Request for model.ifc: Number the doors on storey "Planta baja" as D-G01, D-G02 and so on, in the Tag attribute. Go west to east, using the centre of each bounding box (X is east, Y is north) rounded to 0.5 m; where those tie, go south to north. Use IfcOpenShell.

First a look at what the model holds.

```python
import ifcopenshell
import ifcopenshell.util.element
import ifcopenshell.util.placement

model = ifcopenshell.open("model.ifc")
print(model.schema)
storey = next(s for s in model.by_type("IfcBuildingStorey") if s.Name == "Planta baja")
doors = [e for e in ifcopenshell.util.element.get_decomposition(storey) if e.is_a("IfcDoor")]
for e in sorted(doors, key=lambda e: e.id()):
    origin = ifcopenshell.util.placement.get_local_placement(e.ObjectPlacement)[:3, 3]
    print(e.id(), e.Tag, e.Name, origin.round(2) + 0.0, sep=" | ")
```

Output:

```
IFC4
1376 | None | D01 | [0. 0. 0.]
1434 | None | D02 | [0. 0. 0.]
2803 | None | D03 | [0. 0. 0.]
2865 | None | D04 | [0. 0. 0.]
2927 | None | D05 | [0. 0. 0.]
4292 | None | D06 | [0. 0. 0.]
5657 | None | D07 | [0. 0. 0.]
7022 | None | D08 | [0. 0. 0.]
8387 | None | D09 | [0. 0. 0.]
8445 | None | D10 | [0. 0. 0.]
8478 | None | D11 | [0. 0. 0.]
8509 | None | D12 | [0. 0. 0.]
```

```python
import ifcopenshell
import ifcopenshell.geom
import ifcopenshell.util.element
import ifcopenshell.util.shape

model = ifcopenshell.open("model.ifc")
settings = ifcopenshell.geom.settings()
settings.set("use-world-coords", True)


def centre(element):
    shape = ifcopenshell.geom.create_shape(settings, element)
    return ifcopenshell.util.shape.get_bbox_centroid(shape.geometry)


storey = next(s for s in model.by_type("IfcBuildingStorey") if s.Name == "Planta baja")
doors = [e for e in ifcopenshell.util.element.get_decomposition(storey) if e.is_a("IfcDoor")]

# Insertion points can sit at a corner or the storey origin, so sort by the geometry (in metres).
centres = {e: centre(e) for e in doors}
doors.sort(key=lambda e: (round(centres[e][0] / 0.5), centres[e][1]))

for i, e in enumerate(doors, start=1):
    number = f"D-G{i:02d}"
    e.Tag = number
    print(e.id(), number)

model.write("model_edited.ifc")
```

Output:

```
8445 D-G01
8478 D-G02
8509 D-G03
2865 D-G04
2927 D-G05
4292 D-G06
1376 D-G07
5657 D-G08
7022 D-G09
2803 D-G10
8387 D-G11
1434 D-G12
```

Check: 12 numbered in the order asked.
